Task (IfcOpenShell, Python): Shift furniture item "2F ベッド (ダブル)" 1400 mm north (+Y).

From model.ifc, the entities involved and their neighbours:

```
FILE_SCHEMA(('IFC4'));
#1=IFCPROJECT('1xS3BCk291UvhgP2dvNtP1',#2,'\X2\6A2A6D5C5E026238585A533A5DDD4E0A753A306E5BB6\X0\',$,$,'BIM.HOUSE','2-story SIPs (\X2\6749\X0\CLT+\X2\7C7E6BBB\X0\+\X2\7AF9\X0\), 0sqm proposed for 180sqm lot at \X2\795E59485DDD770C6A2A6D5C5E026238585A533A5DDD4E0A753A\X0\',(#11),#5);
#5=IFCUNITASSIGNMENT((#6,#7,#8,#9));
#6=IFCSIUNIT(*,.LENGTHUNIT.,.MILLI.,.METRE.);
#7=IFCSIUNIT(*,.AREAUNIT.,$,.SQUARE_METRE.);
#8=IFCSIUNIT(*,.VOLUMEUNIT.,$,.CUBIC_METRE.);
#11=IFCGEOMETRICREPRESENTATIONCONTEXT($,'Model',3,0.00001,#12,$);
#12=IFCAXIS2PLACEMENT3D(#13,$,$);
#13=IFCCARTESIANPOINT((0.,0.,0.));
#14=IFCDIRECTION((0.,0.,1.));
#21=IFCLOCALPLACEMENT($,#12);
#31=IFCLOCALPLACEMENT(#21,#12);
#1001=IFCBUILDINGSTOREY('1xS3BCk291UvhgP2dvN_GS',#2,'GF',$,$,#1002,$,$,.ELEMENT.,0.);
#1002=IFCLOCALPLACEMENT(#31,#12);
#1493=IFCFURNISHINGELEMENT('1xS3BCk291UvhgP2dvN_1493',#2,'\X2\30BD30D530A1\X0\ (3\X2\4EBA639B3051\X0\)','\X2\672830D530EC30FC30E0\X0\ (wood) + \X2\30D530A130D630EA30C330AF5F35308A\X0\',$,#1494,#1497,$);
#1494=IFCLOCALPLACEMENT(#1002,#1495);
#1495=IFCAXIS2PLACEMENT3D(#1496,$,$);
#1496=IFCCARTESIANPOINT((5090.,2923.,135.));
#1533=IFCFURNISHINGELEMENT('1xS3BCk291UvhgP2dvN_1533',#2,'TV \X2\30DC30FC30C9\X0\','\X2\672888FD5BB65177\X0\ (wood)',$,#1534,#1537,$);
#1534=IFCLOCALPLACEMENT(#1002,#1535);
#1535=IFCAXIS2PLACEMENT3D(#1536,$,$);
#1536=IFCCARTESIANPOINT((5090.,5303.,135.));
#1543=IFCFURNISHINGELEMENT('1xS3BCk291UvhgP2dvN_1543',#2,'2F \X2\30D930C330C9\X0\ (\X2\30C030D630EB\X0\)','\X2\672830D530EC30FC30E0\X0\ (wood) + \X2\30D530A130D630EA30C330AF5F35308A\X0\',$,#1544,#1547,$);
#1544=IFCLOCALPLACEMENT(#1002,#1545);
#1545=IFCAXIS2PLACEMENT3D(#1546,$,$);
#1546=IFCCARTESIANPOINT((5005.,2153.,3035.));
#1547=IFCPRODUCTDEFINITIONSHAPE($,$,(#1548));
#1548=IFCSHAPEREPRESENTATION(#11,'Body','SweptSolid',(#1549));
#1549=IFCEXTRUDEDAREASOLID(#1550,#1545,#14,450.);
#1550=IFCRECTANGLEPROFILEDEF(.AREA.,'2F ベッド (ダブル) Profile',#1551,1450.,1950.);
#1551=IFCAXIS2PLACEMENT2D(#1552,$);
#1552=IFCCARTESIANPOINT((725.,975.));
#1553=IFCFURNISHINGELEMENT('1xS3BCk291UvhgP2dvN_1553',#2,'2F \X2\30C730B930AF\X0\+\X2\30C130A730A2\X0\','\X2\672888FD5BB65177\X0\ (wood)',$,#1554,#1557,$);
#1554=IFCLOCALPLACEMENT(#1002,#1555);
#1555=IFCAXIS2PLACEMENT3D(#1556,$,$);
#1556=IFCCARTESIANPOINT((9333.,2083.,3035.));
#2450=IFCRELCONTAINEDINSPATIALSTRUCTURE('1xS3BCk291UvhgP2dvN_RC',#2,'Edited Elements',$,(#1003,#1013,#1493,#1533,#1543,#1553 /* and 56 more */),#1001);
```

```python
import ifcopenshell
import ifcopenshell.api.geometry
import ifcopenshell.util.placement
import ifcopenshell.util.unit

model = ifcopenshell.open("model.ifc")
unit_scale = ifcopenshell.util.unit.calculate_unit_scale(model)

item = model.by_guid("1xS3BCk291UvhgP2dvN_1543")
matrix = ifcopenshell.util.placement.get_local_placement(item.ObjectPlacement)
matrix[1, 3] += 1.4 / unit_scale
ifcopenshell.api.geometry.edit_object_placement(model, product=item, matrix=matrix, is_si=False)

print(ifcopenshell.util.placement.get_local_placement(item.ObjectPlacement).round(3) + 0.0)

model.write("model-out.ifc")
```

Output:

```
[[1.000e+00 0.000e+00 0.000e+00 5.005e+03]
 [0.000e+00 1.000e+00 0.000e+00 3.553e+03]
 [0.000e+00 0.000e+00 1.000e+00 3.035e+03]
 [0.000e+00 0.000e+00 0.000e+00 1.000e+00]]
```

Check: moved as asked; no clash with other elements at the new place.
